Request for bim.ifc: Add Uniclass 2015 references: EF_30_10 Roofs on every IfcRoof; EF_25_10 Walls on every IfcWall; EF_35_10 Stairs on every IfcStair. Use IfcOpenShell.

First a look at what the model holds.

```python
import ifcopenshell

model = ifcopenshell.open("bim.ifc")
print(model.schema)
print("classifications:", [c.Name for c in model.by_type("IfcClassification")])
for ifc_class in ("IfcDoor", "IfcRoof", "IfcStair", "IfcWall", "IfcWindow"):
    print(ifc_class, len(model.by_type(ifc_class)))
```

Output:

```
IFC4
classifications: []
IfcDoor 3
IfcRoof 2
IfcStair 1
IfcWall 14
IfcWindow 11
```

```python
import ifcopenshell
import ifcopenshell.api.classification

model = ifcopenshell.open("bim.ifc")

system = ifcopenshell.api.classification.add_classification(model, classification="Uniclass 2015")

codes = {
    "IfcRoof": ("EF_30_10", "Roofs"),
    "IfcWall": ("EF_25_10", "Walls"),
    "IfcStair": ("EF_35_10", "Stairs"),
}
for ifc_class, (code, name) in codes.items():
    products = model.by_type(ifc_class)
    ifcopenshell.api.classification.add_reference(
        model, products=products, classification=system, identification=code, name=name
    )
    print(code, len(products))

model.write("bim_rev.ifc")
```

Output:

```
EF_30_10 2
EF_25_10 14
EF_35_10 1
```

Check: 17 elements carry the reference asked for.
